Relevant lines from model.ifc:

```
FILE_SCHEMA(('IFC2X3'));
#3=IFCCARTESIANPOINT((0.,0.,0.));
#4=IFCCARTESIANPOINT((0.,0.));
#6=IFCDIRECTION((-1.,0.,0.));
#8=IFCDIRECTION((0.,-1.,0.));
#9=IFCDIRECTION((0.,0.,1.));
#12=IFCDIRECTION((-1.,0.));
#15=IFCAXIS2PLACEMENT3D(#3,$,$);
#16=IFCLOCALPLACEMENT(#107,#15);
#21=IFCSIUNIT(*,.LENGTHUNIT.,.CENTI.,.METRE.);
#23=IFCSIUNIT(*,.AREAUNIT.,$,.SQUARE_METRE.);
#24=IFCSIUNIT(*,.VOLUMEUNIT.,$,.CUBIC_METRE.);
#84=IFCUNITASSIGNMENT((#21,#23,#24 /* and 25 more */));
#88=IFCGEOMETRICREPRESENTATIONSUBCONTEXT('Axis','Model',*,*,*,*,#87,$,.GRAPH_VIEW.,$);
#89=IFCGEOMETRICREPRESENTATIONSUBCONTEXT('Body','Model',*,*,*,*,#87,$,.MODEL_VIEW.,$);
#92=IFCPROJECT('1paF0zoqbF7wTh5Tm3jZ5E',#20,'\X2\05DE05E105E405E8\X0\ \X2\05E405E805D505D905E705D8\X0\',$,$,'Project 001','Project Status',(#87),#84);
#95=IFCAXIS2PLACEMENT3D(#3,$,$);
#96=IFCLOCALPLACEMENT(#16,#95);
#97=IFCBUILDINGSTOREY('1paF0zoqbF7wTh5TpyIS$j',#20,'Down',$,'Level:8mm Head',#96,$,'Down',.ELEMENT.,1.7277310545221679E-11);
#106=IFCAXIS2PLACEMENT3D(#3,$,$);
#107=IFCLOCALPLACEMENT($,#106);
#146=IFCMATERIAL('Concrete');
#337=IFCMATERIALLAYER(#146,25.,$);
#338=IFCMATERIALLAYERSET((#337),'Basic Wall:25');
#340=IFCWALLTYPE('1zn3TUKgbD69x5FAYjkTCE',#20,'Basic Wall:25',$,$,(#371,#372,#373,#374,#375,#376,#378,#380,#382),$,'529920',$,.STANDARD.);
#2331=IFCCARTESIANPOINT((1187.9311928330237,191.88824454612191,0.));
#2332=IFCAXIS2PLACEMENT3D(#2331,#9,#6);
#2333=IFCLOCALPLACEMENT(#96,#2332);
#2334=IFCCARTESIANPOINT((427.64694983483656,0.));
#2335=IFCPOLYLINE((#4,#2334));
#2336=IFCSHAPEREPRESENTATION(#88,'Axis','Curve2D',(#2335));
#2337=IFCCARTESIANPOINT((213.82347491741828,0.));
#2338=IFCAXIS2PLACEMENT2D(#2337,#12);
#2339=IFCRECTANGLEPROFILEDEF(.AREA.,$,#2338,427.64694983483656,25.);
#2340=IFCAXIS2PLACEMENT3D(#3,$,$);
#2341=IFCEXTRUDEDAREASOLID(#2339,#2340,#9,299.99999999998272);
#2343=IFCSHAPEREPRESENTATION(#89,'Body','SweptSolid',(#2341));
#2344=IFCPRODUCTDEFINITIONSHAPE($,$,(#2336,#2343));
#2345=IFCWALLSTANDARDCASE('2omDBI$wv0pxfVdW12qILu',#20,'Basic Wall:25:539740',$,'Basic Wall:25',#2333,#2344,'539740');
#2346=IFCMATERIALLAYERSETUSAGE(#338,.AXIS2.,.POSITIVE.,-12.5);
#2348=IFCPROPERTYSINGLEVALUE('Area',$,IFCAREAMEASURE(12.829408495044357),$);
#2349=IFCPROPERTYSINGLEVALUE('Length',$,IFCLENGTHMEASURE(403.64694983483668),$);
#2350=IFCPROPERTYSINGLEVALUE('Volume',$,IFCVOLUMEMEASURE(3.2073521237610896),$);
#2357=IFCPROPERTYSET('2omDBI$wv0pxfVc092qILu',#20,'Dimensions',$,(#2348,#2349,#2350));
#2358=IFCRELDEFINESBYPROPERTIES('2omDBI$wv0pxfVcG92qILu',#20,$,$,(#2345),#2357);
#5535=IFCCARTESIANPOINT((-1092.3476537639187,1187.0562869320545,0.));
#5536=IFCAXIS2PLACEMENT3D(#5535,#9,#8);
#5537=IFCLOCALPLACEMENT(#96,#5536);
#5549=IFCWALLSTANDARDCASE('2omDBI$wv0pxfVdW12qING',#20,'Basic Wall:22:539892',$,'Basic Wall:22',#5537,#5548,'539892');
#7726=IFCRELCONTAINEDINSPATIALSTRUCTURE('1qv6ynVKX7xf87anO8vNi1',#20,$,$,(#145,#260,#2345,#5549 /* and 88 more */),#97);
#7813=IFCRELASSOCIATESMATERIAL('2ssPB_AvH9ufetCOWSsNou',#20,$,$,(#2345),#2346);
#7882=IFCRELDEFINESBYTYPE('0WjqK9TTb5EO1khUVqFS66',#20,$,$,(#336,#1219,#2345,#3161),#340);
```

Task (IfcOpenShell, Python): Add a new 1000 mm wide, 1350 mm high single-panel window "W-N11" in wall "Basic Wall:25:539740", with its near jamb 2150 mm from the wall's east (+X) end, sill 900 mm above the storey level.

```python
import numpy as np
import ifcopenshell
import ifcopenshell.api.feature
import ifcopenshell.api.geometry
import ifcopenshell.api.pset
import ifcopenshell.api.root
import ifcopenshell.api.spatial
import ifcopenshell.api.type
import ifcopenshell.geom
import ifcopenshell.util.element
import ifcopenshell.util.placement
import ifcopenshell.util.representation
import ifcopenshell.util.shape
import ifcopenshell.util.unit

model = ifcopenshell.open("model.ifc")
unit_scale = ifcopenshell.util.unit.calculate_unit_scale(model)
area_scale = ifcopenshell.util.unit.calculate_unit_scale(model, "AREAUNIT")
volume_scale = ifcopenshell.util.unit.calculate_unit_scale(model, "VOLUMEUNIT")
settings = ifcopenshell.geom.settings()


def volume(element):
    """Net volume in cubic metres, openings subtracted."""
    shape = ifcopenshell.geom.create_shape(settings, element)
    return ifcopenshell.util.shape.get_volume(shape.geometry)


wall = model.by_guid("2omDBI$wv0pxfVdW12qILu")
storey = ifcopenshell.util.element.get_container(wall, ifc_class="IfcBuildingStorey")
context = ifcopenshell.util.representation.get_context(model, "Model", "Body", "MODEL_VIEW")
before = volume(wall)

width, height, from_end, sill = 1, 1.35, 2.15, 0.9  # metres

# The wall runs along its own X axis, and the end named is its -X end.
wall_shape = ifcopenshell.geom.create_shape(settings, wall)
x, y, z = ifcopenshell.util.shape.get_vertices(wall_shape.geometry).T
start = x.min() + from_end
face, thickness = float(y.min()), float(y.max() - y.min())
wall_matrix = ifcopenshell.util.placement.get_local_placement(wall.ObjectPlacement)
level = ifcopenshell.util.placement.get_local_placement(storey.ObjectPlacement)[2, 3]


def in_wall(x, y):
    """Placement at x, y metres in the wall's axes, at sill height."""
    matrix = wall_matrix.copy()
    matrix[:, 3] = wall_matrix @ np.array([x / unit_scale, y / unit_scale, 0.0, 1.0])
    matrix[2, 3] = level + sill / unit_scale
    return matrix


# Opening: a box that overshoots both wall faces by 50 mm.
opening = ifcopenshell.api.root.create_entity(model, ifc_class="IfcOpeningElement")
box = ifcopenshell.api.geometry.add_wall_representation(
    model, context=context, length=width, height=height, thickness=thickness + 0.1
)
ifcopenshell.api.geometry.assign_representation(model, product=opening, representation=box)
ifcopenshell.api.geometry.edit_object_placement(model, product=opening, matrix=in_wall(start, face - 0.05), is_si=False)
ifcopenshell.api.feature.add_feature(model, feature=opening, element=wall)

window = ifcopenshell.api.root.create_entity(model, ifc_class="IfcWindow", name="W-N11")
window.OverallWidth, window.OverallHeight = width / unit_scale, height / unit_scale
body = ifcopenshell.api.geometry.add_window_representation(
    model,
    context=context,
    overall_width=window.OverallWidth,
    overall_height=window.OverallHeight,
    partition_type="SINGLE_PANEL",
)
ifcopenshell.api.geometry.assign_representation(model, product=window, representation=body)
ifcopenshell.api.spatial.assign_container(model, products=[window], relating_structure=storey)
fills = ifcopenshell.api.feature.add_filling(model, opening=opening, element=window)
fills.OwnerHistory = window.OwnerHistory  # required in IFC2X3

# IFC2X3 keeps the operation on the window style.
style = ifcopenshell.api.root.create_entity(model, ifc_class="IfcWindowStyle", name="W-N11")
style.OperationType, style.ConstructionType = "SINGLE_PANEL", "NOTDEFINED"
style.ParameterTakesPrecedence = style.Sizeable = False
ifcopenshell.api.type.assign_type(model, related_objects=[window], relating_type=style)

# Centre the window in the wall's thickness.
ifcopenshell.api.geometry.edit_object_placement(model, product=window, matrix=in_wall(start, face), is_si=False)
window_shape = ifcopenshell.geom.create_shape(settings, window)
depth = ifcopenshell.util.shape.get_vertices(window_shape.geometry)[:, 1]
offset = face + thickness / 2 - (depth.min() + depth.max()) / 2
ifcopenshell.api.geometry.edit_object_placement(model, product=window, matrix=in_wall(start, offset), is_si=False)

after = volume(wall)

# Update the wall's stored quantities.
pset = model.by_id(ifcopenshell.util.element.get_pset(wall, "Dimensions", should_inherit=False)["id"])
ifcopenshell.api.pset.edit_pset(model, pset=pset, properties={
    "Area": model.create_entity("IfcAreaMeasure", after / thickness / area_scale),
    "Volume": model.create_entity("IfcVolumeMeasure", after / volume_scale),
})

print(f"wall volume {before:.3f} -> {after:.3f} m3")

model.write("model_updated.ifc")
```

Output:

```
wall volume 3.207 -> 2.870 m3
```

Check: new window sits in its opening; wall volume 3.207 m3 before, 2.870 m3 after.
